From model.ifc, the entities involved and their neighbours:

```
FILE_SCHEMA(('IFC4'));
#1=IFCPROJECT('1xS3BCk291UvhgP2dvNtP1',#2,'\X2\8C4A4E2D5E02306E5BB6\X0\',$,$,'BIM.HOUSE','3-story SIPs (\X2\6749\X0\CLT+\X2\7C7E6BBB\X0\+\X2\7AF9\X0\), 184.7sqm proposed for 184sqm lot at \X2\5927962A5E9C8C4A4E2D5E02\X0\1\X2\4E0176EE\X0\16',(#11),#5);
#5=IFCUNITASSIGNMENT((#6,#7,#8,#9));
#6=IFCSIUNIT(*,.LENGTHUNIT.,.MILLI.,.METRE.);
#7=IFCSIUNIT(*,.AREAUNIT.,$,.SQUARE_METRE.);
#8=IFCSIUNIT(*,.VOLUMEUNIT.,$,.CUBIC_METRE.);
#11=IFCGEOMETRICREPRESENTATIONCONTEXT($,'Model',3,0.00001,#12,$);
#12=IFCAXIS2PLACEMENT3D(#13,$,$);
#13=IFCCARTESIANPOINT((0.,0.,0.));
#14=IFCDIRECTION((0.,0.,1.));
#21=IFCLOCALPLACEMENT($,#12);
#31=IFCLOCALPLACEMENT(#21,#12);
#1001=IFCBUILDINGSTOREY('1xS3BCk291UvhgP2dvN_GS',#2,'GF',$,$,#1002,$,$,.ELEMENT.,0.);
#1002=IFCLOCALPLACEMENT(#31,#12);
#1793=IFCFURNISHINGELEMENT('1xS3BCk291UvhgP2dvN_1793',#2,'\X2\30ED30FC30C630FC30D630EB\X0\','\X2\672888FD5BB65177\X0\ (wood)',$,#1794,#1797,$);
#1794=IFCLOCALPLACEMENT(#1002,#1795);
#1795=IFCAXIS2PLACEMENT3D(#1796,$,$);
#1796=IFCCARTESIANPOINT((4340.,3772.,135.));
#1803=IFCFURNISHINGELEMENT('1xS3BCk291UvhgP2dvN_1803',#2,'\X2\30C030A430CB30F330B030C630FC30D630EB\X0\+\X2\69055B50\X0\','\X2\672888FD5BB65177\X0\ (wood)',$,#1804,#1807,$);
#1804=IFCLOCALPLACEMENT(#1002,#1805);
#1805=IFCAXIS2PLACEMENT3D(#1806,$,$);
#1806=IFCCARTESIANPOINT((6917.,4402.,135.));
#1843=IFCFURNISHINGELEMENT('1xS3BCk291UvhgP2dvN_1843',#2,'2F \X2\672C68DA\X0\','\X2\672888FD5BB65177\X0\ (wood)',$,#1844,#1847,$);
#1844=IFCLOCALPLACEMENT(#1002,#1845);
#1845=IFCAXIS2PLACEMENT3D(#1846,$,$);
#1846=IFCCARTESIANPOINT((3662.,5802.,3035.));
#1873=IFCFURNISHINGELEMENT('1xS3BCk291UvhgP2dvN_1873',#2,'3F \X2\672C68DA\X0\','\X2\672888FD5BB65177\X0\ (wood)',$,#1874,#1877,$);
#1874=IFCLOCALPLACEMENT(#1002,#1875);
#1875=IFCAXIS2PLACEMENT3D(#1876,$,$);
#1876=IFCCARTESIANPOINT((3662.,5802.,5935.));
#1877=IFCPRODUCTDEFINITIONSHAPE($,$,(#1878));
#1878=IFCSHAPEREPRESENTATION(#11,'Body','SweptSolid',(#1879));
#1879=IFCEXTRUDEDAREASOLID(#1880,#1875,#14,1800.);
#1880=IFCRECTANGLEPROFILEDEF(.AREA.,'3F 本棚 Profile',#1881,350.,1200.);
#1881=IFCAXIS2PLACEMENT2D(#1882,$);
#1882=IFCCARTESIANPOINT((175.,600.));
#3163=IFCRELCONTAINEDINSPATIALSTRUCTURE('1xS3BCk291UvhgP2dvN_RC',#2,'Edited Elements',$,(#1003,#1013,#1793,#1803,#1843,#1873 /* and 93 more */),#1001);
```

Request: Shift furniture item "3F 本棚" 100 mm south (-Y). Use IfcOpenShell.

```python
import ifcopenshell
import ifcopenshell.api.geometry
import ifcopenshell.util.placement
import ifcopenshell.util.unit

model = ifcopenshell.open("model.ifc")
unit_scale = ifcopenshell.util.unit.calculate_unit_scale(model)

item = model.by_guid("1xS3BCk291UvhgP2dvN_1873")
matrix = ifcopenshell.util.placement.get_local_placement(item.ObjectPlacement)
matrix[1, 3] -= 0.1 / unit_scale
ifcopenshell.api.geometry.edit_object_placement(model, product=item, matrix=matrix, is_si=False)

print(ifcopenshell.util.placement.get_local_placement(item.ObjectPlacement).round(3) + 0.0)

model.write("model-out.ifc")
```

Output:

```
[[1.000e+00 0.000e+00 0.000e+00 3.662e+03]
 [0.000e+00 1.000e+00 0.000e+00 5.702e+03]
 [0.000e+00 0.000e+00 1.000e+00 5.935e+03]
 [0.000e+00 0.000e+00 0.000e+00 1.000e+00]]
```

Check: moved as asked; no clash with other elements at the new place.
